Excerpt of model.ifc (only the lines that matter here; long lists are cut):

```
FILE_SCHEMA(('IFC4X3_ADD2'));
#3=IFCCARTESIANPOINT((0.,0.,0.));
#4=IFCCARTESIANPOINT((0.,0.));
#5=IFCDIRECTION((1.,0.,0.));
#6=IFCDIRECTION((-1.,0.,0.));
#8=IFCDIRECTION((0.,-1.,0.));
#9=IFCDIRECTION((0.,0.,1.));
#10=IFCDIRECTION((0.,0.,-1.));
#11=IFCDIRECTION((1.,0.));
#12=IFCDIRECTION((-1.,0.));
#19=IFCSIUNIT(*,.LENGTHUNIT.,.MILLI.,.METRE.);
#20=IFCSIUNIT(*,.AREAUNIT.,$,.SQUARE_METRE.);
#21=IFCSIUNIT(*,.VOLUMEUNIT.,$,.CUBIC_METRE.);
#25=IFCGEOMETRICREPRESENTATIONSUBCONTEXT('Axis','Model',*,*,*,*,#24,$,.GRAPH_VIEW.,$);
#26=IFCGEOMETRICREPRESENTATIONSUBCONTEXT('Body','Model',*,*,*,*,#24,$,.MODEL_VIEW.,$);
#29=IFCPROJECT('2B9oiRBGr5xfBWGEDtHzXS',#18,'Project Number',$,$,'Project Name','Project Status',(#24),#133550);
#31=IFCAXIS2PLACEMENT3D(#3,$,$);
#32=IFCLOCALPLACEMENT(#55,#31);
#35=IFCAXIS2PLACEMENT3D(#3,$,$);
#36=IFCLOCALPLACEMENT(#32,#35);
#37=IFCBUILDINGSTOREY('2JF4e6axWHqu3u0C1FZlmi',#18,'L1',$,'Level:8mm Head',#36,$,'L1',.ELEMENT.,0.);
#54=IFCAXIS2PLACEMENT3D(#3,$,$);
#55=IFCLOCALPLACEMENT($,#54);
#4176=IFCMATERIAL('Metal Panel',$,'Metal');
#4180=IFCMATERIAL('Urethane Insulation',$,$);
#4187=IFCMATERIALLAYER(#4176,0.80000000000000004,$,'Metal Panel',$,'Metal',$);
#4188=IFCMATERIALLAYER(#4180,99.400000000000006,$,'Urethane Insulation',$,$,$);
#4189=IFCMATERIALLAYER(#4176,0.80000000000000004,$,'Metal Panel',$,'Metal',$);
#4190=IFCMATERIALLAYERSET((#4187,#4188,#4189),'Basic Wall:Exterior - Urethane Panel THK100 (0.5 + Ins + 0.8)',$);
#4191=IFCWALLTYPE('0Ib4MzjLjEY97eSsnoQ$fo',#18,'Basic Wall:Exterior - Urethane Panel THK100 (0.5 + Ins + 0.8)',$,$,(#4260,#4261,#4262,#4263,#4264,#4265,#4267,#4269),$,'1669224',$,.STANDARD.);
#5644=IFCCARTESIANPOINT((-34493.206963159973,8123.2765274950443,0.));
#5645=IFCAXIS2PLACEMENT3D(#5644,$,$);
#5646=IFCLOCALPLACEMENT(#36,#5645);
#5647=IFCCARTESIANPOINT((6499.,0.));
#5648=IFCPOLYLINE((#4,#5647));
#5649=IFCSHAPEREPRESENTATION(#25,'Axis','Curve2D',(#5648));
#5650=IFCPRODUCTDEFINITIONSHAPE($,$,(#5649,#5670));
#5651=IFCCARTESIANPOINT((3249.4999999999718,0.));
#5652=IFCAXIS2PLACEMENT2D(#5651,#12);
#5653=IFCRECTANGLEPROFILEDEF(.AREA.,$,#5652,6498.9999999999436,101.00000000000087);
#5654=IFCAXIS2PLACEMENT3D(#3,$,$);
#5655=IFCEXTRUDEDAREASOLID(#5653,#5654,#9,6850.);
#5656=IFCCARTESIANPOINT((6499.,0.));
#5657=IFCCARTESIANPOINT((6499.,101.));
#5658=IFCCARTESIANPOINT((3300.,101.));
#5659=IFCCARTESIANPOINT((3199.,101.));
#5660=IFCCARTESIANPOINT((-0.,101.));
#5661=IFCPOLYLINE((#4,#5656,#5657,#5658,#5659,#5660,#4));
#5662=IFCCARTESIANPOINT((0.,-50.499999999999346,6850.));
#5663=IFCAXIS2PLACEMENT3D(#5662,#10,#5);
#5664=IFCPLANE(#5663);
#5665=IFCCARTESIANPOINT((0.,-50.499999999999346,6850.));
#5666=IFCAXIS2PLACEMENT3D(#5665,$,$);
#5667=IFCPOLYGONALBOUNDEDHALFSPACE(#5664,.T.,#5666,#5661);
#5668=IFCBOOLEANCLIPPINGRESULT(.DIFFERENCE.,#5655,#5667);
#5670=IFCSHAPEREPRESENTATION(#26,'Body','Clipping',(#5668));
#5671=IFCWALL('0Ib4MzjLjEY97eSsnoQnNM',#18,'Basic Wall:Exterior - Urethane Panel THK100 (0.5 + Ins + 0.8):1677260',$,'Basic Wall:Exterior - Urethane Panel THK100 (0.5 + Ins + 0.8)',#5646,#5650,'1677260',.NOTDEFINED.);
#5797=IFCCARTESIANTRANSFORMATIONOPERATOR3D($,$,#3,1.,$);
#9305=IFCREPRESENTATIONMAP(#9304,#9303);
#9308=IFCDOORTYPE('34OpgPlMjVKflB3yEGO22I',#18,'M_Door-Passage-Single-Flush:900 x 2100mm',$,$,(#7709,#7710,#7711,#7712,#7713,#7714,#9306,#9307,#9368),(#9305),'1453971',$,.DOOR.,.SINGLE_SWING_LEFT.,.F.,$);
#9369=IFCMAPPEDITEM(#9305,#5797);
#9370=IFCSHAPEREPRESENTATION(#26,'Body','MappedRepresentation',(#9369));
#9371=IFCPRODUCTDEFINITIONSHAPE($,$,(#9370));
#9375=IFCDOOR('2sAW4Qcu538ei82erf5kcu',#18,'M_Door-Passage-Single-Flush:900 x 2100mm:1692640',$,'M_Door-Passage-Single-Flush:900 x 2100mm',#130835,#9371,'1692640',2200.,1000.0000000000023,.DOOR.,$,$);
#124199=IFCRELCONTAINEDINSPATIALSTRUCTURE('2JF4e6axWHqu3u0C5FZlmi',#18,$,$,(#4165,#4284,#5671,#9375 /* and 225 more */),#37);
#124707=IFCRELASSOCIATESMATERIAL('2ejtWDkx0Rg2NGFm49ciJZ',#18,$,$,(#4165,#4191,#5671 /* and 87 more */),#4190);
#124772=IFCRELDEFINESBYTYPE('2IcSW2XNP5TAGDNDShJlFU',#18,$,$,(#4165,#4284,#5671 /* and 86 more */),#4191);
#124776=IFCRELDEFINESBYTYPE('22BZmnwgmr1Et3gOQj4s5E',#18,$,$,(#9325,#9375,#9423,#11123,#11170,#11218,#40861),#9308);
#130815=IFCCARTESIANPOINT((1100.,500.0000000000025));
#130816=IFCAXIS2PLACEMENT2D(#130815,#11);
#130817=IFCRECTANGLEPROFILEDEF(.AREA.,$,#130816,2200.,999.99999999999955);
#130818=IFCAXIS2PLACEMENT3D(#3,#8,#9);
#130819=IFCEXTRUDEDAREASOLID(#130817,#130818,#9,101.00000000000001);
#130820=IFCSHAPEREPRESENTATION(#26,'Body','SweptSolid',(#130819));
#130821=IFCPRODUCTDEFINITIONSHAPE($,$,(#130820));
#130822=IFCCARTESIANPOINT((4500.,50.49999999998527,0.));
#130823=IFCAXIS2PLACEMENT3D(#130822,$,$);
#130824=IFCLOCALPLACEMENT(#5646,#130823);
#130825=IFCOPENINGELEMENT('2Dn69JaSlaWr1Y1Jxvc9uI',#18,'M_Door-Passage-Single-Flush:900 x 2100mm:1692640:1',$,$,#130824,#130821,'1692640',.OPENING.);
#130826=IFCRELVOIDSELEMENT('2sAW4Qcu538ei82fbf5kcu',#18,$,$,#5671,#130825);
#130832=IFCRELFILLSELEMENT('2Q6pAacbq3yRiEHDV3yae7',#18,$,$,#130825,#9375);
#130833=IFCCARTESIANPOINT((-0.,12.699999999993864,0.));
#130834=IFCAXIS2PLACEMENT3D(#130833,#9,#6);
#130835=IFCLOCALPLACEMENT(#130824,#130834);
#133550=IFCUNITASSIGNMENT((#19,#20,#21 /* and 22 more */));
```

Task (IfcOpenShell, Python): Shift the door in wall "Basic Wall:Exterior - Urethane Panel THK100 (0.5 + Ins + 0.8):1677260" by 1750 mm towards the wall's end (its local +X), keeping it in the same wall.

```python
import ifcopenshell
import ifcopenshell.api.geometry
import ifcopenshell.util.placement
import ifcopenshell.util.unit

model = ifcopenshell.open("model.ifc")
unit_scale = ifcopenshell.util.unit.calculate_unit_scale(model)

door = model.by_id(9375)
opening = door.FillsVoids[0].RelatingOpeningElement
wall = opening.VoidsElements[0].RelatingBuildingElement

wall_matrix = ifcopenshell.util.placement.get_local_placement(wall.ObjectPlacement)
shift = wall_matrix[:3, 0] * 1.75 / unit_scale
before = ifcopenshell.util.placement.get_local_placement(door.ObjectPlacement)[:3, 3].copy()

# The door is placed relative to its opening, so it follows when the opening moves.
matrix = ifcopenshell.util.placement.get_local_placement(opening.ObjectPlacement)
matrix[:3, 3] += shift
ifcopenshell.api.geometry.edit_object_placement(
    model, product=opening, matrix=matrix, is_si=False, should_transform_children=True
)

after = ifcopenshell.util.placement.get_local_placement(door.ObjectPlacement)[:3, 3]
print("door moved by", (after - before).round(3) + 0.0)

model.write("model-out.ifc")
```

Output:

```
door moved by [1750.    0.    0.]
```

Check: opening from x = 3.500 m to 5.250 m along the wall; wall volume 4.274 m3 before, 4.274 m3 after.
